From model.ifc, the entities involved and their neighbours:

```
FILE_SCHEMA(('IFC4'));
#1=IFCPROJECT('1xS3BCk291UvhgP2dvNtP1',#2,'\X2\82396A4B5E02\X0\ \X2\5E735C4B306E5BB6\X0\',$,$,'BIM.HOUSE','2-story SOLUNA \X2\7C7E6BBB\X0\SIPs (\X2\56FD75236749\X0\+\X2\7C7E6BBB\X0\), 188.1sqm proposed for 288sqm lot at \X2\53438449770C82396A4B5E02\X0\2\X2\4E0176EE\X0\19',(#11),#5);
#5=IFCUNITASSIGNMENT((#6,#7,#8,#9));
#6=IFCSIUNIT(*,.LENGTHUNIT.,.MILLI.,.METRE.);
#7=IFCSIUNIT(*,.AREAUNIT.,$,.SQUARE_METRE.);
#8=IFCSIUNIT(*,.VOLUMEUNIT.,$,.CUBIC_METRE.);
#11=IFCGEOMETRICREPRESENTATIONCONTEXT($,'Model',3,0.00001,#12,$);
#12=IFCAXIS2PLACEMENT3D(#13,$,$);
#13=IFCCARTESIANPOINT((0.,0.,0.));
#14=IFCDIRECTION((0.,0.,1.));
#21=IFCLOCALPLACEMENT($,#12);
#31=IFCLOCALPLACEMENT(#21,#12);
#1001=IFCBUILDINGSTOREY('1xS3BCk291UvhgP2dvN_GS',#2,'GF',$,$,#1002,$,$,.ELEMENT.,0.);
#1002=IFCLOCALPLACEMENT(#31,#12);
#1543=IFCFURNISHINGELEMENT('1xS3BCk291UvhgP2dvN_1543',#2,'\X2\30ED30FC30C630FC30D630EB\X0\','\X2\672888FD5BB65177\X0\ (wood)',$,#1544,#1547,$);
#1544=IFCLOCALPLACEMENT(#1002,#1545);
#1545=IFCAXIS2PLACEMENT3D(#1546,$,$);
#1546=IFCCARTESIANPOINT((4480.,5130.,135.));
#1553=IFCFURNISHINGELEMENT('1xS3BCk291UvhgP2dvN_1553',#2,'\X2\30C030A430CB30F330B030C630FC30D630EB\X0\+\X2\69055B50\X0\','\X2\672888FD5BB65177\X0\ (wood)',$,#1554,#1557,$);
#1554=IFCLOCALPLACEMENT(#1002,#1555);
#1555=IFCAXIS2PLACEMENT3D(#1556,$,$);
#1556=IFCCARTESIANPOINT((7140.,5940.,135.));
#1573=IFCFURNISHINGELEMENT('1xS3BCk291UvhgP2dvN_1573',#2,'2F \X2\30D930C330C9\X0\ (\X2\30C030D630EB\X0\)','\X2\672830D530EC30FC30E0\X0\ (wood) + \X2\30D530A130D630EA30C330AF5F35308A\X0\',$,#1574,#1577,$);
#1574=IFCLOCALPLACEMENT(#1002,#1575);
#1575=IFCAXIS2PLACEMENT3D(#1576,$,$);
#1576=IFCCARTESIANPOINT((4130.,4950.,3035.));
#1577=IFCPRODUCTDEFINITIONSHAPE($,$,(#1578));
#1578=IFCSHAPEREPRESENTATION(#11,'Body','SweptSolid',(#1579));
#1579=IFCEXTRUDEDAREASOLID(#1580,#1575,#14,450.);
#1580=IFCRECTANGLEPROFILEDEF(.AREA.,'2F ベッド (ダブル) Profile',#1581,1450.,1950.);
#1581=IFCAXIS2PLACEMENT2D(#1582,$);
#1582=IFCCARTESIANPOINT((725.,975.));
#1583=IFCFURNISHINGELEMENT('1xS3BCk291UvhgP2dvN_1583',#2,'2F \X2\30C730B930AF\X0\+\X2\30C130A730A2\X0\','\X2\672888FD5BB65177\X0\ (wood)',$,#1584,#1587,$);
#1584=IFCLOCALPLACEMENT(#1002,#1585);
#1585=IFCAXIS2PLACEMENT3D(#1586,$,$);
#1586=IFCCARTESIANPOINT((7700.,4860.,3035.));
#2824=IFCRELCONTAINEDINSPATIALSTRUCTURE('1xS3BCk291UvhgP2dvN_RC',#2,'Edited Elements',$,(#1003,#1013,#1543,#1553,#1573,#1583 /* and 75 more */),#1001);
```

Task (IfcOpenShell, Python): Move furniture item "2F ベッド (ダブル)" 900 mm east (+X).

```python
import ifcopenshell
import ifcopenshell.api.geometry
import ifcopenshell.util.placement

model = ifcopenshell.open("model.ifc")

item = model.by_guid("1xS3BCk291UvhgP2dvN_1573")
matrix = ifcopenshell.util.placement.get_local_placement(item.ObjectPlacement)
matrix[0, 3] += 900.0
ifcopenshell.api.geometry.edit_object_placement(model, product=item, matrix=matrix, is_si=False)

print(ifcopenshell.util.placement.get_local_placement(item.ObjectPlacement).round(3) + 0.0)

model.write("model_v2.ifc")
```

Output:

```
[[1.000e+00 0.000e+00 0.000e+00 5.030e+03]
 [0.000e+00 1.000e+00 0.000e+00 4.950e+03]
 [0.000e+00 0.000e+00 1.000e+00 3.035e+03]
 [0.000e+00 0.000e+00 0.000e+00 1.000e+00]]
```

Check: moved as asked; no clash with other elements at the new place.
